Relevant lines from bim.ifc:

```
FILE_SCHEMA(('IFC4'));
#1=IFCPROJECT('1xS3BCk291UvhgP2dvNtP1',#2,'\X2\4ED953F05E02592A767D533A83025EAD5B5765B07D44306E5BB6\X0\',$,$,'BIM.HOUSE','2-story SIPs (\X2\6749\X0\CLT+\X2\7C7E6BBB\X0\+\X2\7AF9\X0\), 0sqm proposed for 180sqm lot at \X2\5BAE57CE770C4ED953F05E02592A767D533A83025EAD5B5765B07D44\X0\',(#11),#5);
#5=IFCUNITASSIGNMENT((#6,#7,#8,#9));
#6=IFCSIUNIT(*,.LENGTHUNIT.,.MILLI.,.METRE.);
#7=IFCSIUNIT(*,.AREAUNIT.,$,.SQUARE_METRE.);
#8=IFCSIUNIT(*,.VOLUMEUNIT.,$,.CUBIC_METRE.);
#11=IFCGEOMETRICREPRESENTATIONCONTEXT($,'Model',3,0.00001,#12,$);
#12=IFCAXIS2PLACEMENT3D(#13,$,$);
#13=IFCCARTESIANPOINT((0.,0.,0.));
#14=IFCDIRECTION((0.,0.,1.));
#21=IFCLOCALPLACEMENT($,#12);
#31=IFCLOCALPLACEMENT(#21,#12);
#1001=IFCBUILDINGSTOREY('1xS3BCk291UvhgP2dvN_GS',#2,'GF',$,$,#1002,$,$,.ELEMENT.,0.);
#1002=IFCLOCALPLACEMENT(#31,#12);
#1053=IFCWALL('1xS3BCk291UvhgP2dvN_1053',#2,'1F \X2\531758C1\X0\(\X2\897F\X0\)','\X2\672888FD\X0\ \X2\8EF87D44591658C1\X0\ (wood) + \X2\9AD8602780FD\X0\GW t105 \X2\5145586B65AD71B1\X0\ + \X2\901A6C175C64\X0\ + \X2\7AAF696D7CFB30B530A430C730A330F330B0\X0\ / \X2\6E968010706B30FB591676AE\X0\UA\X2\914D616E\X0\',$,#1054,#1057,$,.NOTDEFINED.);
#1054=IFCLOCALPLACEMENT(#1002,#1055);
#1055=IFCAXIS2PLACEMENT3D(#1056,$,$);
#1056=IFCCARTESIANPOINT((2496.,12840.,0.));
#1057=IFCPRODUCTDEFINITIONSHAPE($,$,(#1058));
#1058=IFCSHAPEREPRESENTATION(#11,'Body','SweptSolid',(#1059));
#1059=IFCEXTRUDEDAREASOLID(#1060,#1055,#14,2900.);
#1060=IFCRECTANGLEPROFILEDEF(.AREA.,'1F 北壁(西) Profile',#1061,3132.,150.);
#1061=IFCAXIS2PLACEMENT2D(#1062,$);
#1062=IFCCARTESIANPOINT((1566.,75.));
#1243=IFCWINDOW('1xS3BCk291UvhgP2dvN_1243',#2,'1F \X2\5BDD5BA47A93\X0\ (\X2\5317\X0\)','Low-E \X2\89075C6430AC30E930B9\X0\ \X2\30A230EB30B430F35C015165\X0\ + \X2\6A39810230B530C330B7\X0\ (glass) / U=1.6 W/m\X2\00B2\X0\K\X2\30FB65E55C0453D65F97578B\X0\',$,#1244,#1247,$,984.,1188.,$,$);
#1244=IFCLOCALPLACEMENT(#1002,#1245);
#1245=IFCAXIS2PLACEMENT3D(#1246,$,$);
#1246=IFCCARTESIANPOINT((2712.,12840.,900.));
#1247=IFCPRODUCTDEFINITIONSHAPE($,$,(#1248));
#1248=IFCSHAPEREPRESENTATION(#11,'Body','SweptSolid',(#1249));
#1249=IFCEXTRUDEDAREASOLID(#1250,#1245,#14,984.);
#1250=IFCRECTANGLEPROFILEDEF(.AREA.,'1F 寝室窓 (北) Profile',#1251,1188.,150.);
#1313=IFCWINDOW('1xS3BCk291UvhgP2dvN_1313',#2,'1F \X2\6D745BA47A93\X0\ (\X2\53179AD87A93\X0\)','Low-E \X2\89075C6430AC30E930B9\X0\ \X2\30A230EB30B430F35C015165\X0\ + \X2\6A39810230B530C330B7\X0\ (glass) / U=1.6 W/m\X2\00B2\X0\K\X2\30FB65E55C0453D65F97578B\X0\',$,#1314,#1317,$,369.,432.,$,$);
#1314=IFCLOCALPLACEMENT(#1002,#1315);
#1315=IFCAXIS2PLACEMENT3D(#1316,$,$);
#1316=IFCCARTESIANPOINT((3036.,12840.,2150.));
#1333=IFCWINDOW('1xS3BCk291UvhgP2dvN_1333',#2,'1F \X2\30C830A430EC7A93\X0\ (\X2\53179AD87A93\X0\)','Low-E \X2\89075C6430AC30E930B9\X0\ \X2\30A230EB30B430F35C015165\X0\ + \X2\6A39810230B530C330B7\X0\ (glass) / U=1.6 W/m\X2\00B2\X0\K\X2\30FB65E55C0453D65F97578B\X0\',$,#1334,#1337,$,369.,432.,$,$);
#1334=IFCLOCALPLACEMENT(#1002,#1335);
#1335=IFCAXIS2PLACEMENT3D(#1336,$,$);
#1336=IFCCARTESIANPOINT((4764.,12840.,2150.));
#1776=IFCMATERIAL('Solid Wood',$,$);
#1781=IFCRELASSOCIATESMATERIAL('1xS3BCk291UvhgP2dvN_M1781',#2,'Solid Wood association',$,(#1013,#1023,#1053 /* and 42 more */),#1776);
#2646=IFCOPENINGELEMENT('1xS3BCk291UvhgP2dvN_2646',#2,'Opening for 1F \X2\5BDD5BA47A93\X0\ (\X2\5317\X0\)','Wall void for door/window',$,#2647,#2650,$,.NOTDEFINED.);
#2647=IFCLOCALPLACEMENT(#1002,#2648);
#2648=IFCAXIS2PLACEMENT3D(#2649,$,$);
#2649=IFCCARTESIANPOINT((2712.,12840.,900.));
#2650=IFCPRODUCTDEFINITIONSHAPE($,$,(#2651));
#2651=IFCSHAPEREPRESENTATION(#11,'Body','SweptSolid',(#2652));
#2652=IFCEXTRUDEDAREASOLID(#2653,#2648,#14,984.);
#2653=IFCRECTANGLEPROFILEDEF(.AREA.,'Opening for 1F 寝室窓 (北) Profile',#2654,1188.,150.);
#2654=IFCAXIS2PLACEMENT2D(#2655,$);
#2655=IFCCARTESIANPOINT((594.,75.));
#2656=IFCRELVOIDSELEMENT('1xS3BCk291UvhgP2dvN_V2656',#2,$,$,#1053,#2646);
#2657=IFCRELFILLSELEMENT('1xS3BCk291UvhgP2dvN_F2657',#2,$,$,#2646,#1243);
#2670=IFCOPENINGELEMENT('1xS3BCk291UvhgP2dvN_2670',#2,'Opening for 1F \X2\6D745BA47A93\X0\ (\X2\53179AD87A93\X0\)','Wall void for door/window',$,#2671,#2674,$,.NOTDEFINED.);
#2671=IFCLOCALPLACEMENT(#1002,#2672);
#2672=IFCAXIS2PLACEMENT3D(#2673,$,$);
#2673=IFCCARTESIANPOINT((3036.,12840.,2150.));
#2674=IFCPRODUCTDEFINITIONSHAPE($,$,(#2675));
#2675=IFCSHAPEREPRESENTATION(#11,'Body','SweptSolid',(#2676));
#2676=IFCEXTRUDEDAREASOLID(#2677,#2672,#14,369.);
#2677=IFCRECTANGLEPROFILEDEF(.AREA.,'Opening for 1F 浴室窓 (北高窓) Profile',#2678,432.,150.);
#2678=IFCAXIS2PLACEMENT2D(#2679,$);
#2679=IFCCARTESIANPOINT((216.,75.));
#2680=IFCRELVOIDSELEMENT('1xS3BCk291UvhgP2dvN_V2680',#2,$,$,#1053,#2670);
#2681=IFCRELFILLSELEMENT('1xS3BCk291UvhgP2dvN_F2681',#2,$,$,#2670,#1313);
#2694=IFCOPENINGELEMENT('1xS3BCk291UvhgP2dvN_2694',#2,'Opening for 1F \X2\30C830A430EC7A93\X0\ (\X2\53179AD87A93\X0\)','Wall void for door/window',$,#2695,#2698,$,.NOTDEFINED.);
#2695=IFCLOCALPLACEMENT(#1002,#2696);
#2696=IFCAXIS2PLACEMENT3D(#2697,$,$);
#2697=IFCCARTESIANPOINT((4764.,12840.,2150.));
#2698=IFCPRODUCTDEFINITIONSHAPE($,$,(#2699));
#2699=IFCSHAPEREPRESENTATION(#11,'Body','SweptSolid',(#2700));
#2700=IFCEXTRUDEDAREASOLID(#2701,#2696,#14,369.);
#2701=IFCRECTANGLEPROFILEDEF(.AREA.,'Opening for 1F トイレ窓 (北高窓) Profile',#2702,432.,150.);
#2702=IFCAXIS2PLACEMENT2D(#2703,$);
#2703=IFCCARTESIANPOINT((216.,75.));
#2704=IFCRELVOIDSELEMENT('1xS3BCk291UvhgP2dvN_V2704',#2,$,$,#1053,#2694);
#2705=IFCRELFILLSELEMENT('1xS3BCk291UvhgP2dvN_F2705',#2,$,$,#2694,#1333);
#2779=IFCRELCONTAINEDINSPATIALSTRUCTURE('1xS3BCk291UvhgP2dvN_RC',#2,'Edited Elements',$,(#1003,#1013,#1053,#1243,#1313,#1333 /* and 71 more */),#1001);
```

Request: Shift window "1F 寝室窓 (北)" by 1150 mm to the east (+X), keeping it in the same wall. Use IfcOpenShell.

```python
import ifcopenshell
import ifcopenshell.api.geometry
import ifcopenshell.util.placement

model = ifcopenshell.open("bim.ifc")

window = model.by_guid("1xS3BCk291UvhgP2dvN_1243")
opening = window.FillsVoids[0].RelatingOpeningElement
wall = opening.VoidsElements[0].RelatingBuildingElement

wall_matrix = ifcopenshell.util.placement.get_local_placement(wall.ObjectPlacement)
shift = wall_matrix[:3, 0] * 1150.0
before = ifcopenshell.util.placement.get_local_placement(window.ObjectPlacement)[:3, 3].copy()

# The window is not placed relative to its opening, so move both.
for product in (opening, window):
    matrix = ifcopenshell.util.placement.get_local_placement(product.ObjectPlacement)
    matrix[:3, 3] += shift
    ifcopenshell.api.geometry.edit_object_placement(model, product=product, matrix=matrix, is_si=False)

after = ifcopenshell.util.placement.get_local_placement(window.ObjectPlacement)[:3, 3]
print("window moved by", (after - before).round(3) + 0.0)

model.write("bim_updated.ifc")
```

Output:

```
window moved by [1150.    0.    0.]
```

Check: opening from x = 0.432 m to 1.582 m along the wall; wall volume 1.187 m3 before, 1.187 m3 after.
